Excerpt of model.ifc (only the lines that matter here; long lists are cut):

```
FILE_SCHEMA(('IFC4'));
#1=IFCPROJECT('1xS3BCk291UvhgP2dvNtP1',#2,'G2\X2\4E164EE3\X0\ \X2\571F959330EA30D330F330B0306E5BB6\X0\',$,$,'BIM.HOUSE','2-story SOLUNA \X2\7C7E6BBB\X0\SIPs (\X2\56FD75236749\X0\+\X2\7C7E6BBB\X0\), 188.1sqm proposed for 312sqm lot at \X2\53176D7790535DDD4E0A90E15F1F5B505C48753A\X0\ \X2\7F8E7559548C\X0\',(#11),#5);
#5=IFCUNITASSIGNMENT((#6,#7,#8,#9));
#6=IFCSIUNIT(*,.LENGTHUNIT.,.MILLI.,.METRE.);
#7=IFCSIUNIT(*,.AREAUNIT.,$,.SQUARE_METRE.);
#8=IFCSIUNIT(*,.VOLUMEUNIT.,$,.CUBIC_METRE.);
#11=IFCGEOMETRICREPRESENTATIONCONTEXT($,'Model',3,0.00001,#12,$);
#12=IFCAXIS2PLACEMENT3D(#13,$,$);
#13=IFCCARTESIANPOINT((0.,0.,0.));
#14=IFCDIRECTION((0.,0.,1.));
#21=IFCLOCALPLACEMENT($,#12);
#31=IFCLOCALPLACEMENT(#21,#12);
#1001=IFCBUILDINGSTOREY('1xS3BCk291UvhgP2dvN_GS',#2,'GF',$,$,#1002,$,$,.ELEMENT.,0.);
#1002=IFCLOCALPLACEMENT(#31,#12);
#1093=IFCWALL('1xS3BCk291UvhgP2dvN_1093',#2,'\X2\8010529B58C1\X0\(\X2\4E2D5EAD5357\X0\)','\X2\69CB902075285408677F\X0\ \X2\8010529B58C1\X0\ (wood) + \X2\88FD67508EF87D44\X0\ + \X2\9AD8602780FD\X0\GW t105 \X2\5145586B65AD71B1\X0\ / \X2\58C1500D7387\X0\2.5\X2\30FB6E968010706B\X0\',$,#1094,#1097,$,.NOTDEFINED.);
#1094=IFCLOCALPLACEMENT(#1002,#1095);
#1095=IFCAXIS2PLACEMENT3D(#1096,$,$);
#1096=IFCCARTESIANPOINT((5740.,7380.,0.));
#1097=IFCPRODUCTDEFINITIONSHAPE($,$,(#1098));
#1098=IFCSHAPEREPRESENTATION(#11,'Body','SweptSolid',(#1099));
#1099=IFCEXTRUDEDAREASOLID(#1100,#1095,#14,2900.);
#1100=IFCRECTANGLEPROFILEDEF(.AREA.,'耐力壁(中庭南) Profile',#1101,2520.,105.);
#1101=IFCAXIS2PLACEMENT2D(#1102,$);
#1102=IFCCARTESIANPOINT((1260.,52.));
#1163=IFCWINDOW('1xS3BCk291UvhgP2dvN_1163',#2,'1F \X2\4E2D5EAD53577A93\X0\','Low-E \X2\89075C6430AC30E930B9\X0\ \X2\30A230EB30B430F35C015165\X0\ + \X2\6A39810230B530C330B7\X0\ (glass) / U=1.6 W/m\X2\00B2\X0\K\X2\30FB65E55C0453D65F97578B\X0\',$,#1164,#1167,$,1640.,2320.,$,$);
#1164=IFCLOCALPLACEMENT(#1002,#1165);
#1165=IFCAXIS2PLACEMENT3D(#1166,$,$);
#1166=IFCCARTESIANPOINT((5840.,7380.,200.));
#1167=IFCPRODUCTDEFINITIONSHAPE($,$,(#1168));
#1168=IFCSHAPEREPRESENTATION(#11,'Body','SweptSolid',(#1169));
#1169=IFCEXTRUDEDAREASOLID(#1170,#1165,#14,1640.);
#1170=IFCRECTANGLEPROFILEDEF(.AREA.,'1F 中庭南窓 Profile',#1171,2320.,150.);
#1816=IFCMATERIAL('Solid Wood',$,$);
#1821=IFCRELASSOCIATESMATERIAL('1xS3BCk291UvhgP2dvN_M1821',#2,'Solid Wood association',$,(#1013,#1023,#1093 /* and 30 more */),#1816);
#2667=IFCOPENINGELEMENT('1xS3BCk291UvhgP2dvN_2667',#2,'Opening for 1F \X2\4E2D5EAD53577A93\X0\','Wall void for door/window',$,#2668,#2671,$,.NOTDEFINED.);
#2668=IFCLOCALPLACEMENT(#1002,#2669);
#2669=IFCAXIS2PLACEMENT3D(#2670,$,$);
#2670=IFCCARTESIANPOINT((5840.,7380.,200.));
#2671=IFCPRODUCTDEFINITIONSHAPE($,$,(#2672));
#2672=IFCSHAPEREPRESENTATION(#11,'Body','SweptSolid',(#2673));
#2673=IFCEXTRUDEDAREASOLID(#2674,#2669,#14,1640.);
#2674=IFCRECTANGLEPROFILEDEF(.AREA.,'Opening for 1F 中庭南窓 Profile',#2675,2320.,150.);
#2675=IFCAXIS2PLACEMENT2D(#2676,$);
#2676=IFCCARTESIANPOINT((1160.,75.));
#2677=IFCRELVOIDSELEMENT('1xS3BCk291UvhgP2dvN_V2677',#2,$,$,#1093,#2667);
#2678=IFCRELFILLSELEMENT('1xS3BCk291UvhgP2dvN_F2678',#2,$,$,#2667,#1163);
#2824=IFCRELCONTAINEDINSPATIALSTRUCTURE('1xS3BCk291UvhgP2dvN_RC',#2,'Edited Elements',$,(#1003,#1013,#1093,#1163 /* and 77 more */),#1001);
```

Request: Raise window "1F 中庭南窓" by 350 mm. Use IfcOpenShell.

```python
import numpy as np
import ifcopenshell
import ifcopenshell.api.geometry
import ifcopenshell.util.placement
import ifcopenshell.util.unit

model = ifcopenshell.open("model.ifc")
unit_scale = ifcopenshell.util.unit.calculate_unit_scale(model)

window = model.by_guid("1xS3BCk291UvhgP2dvN_1163")
opening = window.FillsVoids[0].RelatingOpeningElement
dz = 0.35 / unit_scale

shift = np.array([0.0, 0.0, dz])
# The window is not placed relative to its opening, so move both.
for product in (opening, window):
    matrix = ifcopenshell.util.placement.get_local_placement(product.ObjectPlacement)
    matrix[:3, 3] += shift
    ifcopenshell.api.geometry.edit_object_placement(model, product=product, matrix=matrix, is_si=False)

print(f"moved by {dz * unit_scale:+.3f} m")

model.write("model-out.ifc")
```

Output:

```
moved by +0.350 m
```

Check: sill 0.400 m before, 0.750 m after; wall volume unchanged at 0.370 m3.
